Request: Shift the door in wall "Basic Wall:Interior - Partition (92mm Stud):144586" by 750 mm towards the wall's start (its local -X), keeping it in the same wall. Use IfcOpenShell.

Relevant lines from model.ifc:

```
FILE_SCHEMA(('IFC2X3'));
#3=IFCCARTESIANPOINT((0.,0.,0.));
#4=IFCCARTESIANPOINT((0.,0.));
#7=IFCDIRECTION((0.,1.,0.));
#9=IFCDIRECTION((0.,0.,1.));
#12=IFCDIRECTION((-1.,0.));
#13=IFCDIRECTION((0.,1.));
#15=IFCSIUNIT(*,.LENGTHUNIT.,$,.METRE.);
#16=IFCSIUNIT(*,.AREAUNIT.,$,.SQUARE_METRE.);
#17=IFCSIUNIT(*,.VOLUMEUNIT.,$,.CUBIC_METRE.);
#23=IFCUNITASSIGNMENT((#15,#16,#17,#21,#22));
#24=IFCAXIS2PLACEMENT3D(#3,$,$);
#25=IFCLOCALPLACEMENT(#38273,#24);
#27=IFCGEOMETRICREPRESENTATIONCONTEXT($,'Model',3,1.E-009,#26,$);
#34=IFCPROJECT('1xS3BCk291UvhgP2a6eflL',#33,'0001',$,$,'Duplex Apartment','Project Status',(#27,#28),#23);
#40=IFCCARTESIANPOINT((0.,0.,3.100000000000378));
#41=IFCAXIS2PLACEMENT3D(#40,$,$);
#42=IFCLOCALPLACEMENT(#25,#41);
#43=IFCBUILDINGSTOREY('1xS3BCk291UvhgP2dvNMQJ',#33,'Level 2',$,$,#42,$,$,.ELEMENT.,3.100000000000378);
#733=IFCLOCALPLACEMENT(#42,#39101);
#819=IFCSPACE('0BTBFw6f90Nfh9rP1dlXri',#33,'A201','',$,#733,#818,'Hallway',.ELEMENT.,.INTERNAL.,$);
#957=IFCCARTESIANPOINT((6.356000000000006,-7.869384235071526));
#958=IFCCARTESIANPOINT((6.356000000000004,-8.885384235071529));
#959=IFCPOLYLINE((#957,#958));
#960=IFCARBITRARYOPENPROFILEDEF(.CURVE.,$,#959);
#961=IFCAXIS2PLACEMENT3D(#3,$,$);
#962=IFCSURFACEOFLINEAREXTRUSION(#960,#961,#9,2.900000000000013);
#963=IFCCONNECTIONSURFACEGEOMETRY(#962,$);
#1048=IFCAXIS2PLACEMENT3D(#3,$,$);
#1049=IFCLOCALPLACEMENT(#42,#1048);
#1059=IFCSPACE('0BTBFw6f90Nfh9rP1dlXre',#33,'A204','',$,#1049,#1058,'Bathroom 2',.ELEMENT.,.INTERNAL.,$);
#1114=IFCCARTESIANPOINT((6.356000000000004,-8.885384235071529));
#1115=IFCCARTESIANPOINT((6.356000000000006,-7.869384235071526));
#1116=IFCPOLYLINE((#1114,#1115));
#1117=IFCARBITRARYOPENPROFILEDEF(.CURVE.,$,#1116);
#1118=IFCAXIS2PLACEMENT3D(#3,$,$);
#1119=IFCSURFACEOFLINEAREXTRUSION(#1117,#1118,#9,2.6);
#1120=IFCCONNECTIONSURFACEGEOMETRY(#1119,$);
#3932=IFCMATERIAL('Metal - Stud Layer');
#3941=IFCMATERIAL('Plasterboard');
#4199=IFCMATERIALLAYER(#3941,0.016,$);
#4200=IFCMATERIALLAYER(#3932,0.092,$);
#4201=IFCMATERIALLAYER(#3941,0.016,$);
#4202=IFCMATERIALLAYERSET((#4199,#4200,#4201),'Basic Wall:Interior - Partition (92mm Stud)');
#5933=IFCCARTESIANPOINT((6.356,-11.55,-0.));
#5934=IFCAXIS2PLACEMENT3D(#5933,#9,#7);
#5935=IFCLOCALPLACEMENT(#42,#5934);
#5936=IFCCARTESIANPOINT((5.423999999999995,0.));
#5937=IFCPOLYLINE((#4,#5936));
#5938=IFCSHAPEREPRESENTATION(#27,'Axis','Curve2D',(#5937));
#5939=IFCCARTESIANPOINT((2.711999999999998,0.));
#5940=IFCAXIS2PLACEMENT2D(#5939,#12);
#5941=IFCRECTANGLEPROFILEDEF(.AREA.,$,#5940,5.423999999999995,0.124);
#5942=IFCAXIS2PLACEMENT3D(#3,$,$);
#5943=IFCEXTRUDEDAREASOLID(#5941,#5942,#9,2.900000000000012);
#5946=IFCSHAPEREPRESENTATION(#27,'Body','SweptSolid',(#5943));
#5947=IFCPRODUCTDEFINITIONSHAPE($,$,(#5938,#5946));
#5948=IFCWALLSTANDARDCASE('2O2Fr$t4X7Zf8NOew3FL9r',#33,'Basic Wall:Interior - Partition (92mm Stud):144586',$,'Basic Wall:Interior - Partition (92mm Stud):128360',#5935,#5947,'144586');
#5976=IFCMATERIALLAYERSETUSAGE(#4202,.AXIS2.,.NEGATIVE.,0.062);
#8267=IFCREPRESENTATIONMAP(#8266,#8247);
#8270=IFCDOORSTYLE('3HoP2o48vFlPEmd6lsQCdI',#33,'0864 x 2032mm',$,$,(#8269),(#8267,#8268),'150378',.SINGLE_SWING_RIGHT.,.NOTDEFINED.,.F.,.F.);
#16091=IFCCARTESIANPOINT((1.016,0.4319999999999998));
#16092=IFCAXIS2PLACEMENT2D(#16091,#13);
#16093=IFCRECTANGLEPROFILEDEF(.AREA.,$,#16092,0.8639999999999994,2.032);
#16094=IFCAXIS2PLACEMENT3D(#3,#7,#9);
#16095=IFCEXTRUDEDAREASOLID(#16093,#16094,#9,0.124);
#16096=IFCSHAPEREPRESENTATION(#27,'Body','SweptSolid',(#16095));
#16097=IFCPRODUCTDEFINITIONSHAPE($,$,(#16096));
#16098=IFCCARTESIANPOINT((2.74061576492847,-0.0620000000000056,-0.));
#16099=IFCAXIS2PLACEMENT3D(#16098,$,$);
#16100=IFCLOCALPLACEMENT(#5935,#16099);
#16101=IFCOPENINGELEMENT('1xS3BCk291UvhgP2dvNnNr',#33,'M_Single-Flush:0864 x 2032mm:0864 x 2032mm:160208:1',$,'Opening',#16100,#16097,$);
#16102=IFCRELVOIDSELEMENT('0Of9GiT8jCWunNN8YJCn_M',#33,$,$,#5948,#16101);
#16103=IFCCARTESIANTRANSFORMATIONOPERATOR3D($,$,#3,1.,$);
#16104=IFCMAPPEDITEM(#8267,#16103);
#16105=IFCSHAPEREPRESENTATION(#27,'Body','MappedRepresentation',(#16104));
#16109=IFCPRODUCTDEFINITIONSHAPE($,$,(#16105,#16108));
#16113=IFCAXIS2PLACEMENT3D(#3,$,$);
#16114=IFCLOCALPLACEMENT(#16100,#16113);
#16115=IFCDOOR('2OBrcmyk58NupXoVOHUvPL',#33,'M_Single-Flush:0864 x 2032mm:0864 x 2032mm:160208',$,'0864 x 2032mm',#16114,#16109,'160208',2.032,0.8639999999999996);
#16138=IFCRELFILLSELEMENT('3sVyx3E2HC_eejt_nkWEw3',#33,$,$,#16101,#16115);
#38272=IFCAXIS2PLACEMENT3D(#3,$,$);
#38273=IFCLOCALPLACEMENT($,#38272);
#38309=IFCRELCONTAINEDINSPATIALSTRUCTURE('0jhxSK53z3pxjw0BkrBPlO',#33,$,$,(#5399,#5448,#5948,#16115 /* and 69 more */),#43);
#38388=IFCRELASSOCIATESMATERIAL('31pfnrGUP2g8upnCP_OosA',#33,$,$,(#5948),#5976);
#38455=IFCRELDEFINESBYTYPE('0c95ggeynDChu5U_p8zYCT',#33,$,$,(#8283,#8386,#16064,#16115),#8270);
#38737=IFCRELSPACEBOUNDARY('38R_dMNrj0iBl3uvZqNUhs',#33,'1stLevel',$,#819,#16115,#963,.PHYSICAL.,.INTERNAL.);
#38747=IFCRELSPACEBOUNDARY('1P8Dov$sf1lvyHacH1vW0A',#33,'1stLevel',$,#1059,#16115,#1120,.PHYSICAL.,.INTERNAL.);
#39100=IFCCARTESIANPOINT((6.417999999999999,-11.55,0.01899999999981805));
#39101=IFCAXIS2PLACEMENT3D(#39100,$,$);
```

```python
import numpy as np
import ifcopenshell
import ifcopenshell.api.geometry
import ifcopenshell.util.placement

model = ifcopenshell.open("model.ifc")

door = model.by_id(16115)
opening = door.FillsVoids[0].RelatingOpeningElement
wall = opening.VoidsElements[0].RelatingBuildingElement

wall_matrix = ifcopenshell.util.placement.get_local_placement(wall.ObjectPlacement)
shift = wall_matrix[:3, 0] * -0.75
before = ifcopenshell.util.placement.get_local_placement(door.ObjectPlacement)[:3, 3].copy()

# The door is placed relative to its opening, so it follows when the opening moves.
matrix = ifcopenshell.util.placement.get_local_placement(opening.ObjectPlacement)
matrix[:3, 3] += shift
ifcopenshell.api.geometry.edit_object_placement(
    model, product=opening, matrix=matrix, is_si=False, should_transform_children=True
)

# Space boundary surfaces are stored in each space's coordinates; move them too.
for rel in door.ProvidesBoundaries:
    if not rel.ConnectionGeometry:
        continue
    surface = rel.ConnectionGeometry.SurfaceOnRelatingElement
    space_matrix = ifcopenshell.util.placement.get_local_placement(rel.RelatingSpace.ObjectPlacement)
    point = np.array(surface.Position.Location.Coordinates) + space_matrix[:3, :3].T @ shift
    surface.Position = model.createIfcAxis2Placement3D(
        model.createIfcCartesianPoint(point.tolist()), surface.Position.Axis, surface.Position.RefDirection
    )

after = ifcopenshell.util.placement.get_local_placement(door.ObjectPlacement)[:3, 3]
print("door moved by", (after - before).round(3) + 0.0)

model.write("model_updated.ifc")
```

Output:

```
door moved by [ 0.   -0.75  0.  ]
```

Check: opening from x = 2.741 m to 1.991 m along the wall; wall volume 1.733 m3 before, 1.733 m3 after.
